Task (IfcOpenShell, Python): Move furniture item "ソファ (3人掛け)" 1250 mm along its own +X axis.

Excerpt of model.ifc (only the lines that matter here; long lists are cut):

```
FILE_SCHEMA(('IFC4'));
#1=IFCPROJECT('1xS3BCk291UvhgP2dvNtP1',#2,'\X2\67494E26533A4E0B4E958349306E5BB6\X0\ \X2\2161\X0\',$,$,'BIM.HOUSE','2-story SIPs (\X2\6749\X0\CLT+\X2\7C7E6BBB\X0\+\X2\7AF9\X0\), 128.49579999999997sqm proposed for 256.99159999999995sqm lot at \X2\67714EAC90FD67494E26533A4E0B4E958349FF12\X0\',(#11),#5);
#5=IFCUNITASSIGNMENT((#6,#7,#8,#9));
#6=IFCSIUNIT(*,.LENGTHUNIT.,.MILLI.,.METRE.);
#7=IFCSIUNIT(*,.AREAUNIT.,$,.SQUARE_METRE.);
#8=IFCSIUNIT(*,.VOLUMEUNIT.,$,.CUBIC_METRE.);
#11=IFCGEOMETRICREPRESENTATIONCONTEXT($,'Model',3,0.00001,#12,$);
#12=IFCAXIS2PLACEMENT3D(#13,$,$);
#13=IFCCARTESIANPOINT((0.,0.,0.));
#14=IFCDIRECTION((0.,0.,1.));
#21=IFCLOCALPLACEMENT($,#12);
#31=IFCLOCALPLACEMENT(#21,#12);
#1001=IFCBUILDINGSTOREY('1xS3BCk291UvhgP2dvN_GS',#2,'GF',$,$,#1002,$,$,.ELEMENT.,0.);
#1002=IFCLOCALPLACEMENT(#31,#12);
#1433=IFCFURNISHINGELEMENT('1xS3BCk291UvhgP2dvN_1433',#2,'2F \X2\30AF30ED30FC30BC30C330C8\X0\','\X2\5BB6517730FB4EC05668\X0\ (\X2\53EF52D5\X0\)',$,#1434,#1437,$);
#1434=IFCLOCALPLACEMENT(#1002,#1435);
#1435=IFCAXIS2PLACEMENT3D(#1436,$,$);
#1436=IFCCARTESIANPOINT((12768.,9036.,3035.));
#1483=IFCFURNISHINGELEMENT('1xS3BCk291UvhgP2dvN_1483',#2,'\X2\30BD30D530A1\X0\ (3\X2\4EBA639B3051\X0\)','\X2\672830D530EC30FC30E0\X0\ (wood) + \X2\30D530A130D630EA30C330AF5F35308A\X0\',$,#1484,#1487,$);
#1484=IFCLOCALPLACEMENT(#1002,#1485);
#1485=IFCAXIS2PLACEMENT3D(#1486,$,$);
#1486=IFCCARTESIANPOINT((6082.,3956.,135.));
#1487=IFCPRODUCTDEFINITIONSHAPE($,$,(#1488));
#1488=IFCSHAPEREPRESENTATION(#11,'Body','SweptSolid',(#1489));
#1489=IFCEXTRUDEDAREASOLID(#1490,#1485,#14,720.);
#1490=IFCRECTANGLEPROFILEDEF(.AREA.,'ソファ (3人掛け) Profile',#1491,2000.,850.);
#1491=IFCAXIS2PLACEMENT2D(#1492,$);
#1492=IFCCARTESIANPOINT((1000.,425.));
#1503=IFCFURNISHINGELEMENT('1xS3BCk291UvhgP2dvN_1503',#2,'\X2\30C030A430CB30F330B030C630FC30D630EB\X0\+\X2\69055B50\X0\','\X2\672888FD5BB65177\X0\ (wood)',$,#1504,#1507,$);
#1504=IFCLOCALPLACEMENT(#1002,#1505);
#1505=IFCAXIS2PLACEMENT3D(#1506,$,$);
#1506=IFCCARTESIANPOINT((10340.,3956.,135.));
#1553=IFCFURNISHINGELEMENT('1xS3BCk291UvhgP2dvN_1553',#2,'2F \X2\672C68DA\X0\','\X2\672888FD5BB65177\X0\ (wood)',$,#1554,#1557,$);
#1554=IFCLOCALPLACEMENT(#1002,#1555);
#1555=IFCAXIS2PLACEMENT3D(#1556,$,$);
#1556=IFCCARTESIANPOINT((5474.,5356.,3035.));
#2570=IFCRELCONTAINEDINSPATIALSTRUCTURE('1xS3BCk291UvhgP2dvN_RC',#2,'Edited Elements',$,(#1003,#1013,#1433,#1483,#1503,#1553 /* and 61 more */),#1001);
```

```python
import ifcopenshell
import ifcopenshell.api.geometry
import ifcopenshell.util.placement
import ifcopenshell.util.unit

model = ifcopenshell.open("model.ifc")
unit_scale = ifcopenshell.util.unit.calculate_unit_scale(model)

item = model.by_guid("1xS3BCk291UvhgP2dvN_1483")
matrix = ifcopenshell.util.placement.get_local_placement(item.ObjectPlacement)
matrix[:3, 3] += matrix[:3, 0] * 1.25 / unit_scale
ifcopenshell.api.geometry.edit_object_placement(model, product=item, matrix=matrix, is_si=False)

print(ifcopenshell.util.placement.get_local_placement(item.ObjectPlacement).round(3) + 0.0)

model.write("model_edited.ifc")
```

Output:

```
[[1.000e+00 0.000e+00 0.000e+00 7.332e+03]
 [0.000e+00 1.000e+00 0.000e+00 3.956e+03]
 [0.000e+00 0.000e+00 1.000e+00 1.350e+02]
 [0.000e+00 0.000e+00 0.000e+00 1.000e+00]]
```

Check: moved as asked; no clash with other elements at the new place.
